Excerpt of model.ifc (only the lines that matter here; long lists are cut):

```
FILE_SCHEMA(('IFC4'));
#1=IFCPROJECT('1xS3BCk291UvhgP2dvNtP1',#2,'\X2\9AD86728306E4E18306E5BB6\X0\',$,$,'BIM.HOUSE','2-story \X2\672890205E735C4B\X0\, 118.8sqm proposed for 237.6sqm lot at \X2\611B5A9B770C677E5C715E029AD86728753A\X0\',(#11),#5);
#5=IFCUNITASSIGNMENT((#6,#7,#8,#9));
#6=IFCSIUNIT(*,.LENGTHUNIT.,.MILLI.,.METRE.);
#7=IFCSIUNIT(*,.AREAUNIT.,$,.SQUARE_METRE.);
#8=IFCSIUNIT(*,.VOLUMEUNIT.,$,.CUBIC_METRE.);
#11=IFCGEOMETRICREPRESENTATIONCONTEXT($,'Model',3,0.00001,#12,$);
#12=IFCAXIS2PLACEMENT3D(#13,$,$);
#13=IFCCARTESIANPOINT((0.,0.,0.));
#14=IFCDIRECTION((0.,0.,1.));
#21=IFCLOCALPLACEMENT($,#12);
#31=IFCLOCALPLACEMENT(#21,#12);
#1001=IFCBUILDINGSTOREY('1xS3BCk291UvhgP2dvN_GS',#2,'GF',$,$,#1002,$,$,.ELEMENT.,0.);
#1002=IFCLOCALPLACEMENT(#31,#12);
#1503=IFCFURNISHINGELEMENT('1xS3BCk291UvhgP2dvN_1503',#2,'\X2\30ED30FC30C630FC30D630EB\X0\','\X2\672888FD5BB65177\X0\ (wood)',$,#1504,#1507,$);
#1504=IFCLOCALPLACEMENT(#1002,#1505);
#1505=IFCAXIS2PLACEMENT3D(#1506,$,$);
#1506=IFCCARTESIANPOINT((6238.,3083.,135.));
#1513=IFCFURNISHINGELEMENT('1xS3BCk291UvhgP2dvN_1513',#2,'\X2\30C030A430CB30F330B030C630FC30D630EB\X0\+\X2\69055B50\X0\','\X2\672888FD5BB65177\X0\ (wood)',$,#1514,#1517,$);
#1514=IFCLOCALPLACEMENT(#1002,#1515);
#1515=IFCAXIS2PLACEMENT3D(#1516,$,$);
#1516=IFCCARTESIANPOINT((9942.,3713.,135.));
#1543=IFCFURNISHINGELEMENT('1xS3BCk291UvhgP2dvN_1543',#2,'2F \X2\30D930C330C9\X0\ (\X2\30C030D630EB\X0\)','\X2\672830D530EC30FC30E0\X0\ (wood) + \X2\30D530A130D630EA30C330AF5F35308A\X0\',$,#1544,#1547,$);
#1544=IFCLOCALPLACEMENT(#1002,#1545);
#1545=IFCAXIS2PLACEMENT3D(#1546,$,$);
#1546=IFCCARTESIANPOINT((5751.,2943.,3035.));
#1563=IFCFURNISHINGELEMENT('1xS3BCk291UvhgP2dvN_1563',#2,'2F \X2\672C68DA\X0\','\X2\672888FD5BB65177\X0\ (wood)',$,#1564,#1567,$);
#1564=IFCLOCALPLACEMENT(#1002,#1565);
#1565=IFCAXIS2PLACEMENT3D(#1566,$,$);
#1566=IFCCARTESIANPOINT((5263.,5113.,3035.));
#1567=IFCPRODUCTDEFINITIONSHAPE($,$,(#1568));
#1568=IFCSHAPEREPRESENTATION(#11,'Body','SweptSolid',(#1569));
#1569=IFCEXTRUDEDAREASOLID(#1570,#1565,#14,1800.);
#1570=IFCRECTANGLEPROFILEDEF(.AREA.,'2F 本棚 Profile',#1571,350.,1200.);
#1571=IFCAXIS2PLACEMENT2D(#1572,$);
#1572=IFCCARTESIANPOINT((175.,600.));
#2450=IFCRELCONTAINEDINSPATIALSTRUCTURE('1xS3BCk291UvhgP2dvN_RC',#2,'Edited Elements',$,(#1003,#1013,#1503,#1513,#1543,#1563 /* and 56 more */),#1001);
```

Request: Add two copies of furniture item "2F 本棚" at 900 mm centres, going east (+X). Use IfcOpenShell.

```python
import numpy as np
import ifcopenshell
import ifcopenshell.api.geometry
import ifcopenshell.api.root
import ifcopenshell.util.element
import ifcopenshell.util.placement
import ifcopenshell.util.unit

model = ifcopenshell.open("model.ifc")
unit_scale = ifcopenshell.util.unit.calculate_unit_scale(model)


def reuse_history(source, copy):
    """copy_class also copies each property set's owner history, people and application; keep the originals."""
    for rel in copy.IsDefinedBy:
        if rel.is_a("IfcRelDefinesByProperties") and (history := rel.RelatingPropertyDefinition.OwnerHistory):
            rel.RelatingPropertyDefinition.OwnerHistory = source.OwnerHistory
            ifcopenshell.util.element.remove_deep2(model, history)


source = model.by_guid("1xS3BCk291UvhgP2dvN_1563")
base = ifcopenshell.util.placement.get_local_placement(source.ObjectPlacement)
step = np.array([1.0, 0.0, 0.0]) * 0.9 / unit_scale

for i in range(1, 3):
    copy = ifcopenshell.api.root.copy_class(model, product=source)
    copy.Representation = ifcopenshell.util.element.copy_deep(
        model, source.Representation, exclude=["IfcGeometricRepresentationContext", "IfcRepresentationMap"]
    )
    reuse_history(source, copy)
    matrix = base.copy()
    matrix[:3, 3] += i * step
    print("added at", matrix[:3, 3].round(3) + 0.0)
    ifcopenshell.api.geometry.edit_object_placement(model, product=copy, matrix=matrix, is_si=False)

model.write("model-out.ifc")
```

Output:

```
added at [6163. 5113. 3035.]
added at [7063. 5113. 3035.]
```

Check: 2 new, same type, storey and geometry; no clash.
